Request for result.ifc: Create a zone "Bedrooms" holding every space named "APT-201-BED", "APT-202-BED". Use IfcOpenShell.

First a look at what the model holds.

```python
import ifcopenshell

model = ifcopenshell.open("result.ifc")
print(model.schema)
seen = {}
for space in model.by_type("IfcSpace"):
    seen[space.Name] = seen.get(space.Name, 0) + 1
for name, count in sorted(seen.items(), key=str):
    print(count, "x", name)
print("zones:", [z.Name for z in model.by_type("IfcZone")][:20])
```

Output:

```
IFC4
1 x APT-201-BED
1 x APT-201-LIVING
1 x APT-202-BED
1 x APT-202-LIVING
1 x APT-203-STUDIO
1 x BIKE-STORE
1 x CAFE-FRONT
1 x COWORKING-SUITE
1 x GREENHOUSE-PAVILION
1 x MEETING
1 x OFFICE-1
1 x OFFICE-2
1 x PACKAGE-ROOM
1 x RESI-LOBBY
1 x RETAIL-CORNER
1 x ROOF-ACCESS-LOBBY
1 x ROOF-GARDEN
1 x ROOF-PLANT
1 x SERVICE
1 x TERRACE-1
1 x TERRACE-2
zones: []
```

```python
import ifcopenshell
import ifcopenshell.api.group
import ifcopenshell.api.root

model = ifcopenshell.open("result.ifc")

names = {"APT-201-BED", "APT-202-BED"}
spaces = [s for s in model.by_type("IfcSpace") if s.Name in names]

zone = ifcopenshell.api.root.create_entity(model, ifc_class="IfcZone", name="Bedrooms")
ifcopenshell.api.group.assign_group(model, products=spaces, group=zone)
print(len(spaces), "spaces in", zone.Name)

model.write("result_edited.ifc")
```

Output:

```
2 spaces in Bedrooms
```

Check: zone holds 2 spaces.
